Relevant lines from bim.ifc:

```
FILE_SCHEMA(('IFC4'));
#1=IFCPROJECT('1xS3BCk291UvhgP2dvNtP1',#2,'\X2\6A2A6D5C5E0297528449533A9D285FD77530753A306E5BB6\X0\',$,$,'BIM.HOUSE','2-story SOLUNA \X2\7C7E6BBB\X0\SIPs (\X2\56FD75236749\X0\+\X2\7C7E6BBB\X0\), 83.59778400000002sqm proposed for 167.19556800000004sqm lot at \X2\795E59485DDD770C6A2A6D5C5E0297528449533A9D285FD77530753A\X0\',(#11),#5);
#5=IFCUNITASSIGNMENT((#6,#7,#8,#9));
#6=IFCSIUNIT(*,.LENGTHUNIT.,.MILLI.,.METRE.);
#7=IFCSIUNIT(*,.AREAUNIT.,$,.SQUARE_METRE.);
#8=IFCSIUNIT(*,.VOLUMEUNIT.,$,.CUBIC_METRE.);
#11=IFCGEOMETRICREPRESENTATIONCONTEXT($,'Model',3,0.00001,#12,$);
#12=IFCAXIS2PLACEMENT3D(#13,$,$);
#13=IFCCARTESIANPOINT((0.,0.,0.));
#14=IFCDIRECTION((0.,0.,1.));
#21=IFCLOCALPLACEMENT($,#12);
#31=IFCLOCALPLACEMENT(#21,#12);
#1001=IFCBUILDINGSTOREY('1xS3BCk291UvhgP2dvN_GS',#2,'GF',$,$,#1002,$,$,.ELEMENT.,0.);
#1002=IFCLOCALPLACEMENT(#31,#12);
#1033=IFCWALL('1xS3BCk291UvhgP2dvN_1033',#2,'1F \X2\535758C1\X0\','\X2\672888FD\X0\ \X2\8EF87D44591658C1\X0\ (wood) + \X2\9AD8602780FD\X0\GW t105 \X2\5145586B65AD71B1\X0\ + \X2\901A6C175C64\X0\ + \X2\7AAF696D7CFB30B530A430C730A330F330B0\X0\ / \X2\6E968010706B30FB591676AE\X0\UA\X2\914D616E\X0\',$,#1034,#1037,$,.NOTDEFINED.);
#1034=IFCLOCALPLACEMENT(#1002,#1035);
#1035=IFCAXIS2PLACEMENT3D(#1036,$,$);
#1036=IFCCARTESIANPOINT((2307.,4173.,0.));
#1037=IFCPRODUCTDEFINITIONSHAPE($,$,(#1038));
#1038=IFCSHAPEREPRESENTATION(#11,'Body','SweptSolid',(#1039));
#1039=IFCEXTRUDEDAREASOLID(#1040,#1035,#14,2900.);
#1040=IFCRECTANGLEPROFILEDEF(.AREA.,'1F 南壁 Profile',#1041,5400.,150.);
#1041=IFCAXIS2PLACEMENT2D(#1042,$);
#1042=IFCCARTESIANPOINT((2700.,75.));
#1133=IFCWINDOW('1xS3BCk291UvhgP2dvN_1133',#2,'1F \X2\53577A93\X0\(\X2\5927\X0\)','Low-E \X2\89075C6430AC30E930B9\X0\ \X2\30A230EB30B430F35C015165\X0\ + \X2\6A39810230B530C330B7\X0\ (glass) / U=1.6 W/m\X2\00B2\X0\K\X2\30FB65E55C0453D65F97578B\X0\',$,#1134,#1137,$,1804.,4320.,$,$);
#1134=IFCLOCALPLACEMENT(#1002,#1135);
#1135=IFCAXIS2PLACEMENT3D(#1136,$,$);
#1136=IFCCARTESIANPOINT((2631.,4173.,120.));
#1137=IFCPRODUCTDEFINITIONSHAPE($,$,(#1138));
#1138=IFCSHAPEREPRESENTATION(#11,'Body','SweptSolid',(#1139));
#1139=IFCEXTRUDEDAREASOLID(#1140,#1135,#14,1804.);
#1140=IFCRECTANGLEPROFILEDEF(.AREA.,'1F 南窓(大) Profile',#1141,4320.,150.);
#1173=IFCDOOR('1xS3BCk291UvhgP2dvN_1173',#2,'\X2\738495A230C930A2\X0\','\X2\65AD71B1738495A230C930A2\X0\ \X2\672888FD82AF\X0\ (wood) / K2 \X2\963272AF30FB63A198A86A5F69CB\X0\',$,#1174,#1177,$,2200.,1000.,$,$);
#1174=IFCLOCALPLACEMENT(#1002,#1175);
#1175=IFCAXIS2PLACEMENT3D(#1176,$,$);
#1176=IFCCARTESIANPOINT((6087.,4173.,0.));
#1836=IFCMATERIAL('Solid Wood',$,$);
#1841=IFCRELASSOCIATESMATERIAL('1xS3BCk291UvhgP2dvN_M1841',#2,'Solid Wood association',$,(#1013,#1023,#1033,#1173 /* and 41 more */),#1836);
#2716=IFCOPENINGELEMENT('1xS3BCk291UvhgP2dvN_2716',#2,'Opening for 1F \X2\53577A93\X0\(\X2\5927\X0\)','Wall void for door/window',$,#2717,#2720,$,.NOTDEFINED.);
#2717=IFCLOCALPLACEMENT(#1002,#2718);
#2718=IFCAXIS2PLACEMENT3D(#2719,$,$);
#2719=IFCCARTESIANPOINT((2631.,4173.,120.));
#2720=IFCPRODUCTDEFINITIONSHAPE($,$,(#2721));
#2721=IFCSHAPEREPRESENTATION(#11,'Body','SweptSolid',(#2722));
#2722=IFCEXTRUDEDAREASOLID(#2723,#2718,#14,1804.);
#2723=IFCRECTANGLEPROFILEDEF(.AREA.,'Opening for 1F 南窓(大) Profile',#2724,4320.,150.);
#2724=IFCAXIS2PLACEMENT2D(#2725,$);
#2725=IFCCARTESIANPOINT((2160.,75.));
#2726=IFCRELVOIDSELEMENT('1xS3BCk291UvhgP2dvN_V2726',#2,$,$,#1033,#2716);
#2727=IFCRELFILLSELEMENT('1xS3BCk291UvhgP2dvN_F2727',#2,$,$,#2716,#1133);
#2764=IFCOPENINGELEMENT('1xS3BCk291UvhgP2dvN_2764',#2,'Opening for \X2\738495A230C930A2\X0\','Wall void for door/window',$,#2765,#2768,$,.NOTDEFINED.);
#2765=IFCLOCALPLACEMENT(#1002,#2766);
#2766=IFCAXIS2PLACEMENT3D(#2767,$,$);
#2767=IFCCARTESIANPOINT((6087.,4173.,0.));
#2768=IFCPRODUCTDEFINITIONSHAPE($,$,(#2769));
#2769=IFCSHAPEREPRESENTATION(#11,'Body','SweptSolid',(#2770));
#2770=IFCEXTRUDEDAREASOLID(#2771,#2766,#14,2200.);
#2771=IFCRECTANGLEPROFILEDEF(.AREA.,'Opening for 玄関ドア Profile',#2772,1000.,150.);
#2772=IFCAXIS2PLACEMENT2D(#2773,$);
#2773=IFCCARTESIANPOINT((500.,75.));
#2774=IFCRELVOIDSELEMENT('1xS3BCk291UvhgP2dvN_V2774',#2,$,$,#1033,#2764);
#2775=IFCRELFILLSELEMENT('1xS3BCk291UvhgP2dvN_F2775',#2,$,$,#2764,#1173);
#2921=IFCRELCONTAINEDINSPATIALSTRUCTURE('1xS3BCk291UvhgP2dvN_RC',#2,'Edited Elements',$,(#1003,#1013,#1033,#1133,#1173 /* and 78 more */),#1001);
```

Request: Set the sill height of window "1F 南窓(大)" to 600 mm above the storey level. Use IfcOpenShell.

```python
import numpy as np
import ifcopenshell
import ifcopenshell.api.geometry
import ifcopenshell.geom
import ifcopenshell.util.element
import ifcopenshell.util.placement
import ifcopenshell.util.shape
import ifcopenshell.util.unit

model = ifcopenshell.open("bim.ifc")
unit_scale = ifcopenshell.util.unit.calculate_unit_scale(model)

window = model.by_guid("1xS3BCk291UvhgP2dvN_1133")
opening = window.FillsVoids[0].RelatingOpeningElement
storey = ifcopenshell.util.element.get_container(window, ifc_class="IfcBuildingStorey")
level = ifcopenshell.util.placement.get_local_placement(storey.ObjectPlacement)[2, 3]

# The opening's origin need not be at the sill, so measure its lowest point.
shape = ifcopenshell.geom.create_shape(ifcopenshell.geom.settings(), opening)
bottom = ifcopenshell.util.shape.get_shape_bottom_elevation(shape, shape.geometry) / unit_scale
dz = level + 0.6 / unit_scale - bottom

shift = np.array([0.0, 0.0, dz])
# The window is not placed relative to its opening, so move both.
for product in (opening, window):
    matrix = ifcopenshell.util.placement.get_local_placement(product.ObjectPlacement)
    matrix[:3, 3] += shift
    ifcopenshell.api.geometry.edit_object_placement(model, product=product, matrix=matrix, is_si=False)

print(f"moved by {dz * unit_scale:+.3f} m")

model.write("bim_rev.ifc")
```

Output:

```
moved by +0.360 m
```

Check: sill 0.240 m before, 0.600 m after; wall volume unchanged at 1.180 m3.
